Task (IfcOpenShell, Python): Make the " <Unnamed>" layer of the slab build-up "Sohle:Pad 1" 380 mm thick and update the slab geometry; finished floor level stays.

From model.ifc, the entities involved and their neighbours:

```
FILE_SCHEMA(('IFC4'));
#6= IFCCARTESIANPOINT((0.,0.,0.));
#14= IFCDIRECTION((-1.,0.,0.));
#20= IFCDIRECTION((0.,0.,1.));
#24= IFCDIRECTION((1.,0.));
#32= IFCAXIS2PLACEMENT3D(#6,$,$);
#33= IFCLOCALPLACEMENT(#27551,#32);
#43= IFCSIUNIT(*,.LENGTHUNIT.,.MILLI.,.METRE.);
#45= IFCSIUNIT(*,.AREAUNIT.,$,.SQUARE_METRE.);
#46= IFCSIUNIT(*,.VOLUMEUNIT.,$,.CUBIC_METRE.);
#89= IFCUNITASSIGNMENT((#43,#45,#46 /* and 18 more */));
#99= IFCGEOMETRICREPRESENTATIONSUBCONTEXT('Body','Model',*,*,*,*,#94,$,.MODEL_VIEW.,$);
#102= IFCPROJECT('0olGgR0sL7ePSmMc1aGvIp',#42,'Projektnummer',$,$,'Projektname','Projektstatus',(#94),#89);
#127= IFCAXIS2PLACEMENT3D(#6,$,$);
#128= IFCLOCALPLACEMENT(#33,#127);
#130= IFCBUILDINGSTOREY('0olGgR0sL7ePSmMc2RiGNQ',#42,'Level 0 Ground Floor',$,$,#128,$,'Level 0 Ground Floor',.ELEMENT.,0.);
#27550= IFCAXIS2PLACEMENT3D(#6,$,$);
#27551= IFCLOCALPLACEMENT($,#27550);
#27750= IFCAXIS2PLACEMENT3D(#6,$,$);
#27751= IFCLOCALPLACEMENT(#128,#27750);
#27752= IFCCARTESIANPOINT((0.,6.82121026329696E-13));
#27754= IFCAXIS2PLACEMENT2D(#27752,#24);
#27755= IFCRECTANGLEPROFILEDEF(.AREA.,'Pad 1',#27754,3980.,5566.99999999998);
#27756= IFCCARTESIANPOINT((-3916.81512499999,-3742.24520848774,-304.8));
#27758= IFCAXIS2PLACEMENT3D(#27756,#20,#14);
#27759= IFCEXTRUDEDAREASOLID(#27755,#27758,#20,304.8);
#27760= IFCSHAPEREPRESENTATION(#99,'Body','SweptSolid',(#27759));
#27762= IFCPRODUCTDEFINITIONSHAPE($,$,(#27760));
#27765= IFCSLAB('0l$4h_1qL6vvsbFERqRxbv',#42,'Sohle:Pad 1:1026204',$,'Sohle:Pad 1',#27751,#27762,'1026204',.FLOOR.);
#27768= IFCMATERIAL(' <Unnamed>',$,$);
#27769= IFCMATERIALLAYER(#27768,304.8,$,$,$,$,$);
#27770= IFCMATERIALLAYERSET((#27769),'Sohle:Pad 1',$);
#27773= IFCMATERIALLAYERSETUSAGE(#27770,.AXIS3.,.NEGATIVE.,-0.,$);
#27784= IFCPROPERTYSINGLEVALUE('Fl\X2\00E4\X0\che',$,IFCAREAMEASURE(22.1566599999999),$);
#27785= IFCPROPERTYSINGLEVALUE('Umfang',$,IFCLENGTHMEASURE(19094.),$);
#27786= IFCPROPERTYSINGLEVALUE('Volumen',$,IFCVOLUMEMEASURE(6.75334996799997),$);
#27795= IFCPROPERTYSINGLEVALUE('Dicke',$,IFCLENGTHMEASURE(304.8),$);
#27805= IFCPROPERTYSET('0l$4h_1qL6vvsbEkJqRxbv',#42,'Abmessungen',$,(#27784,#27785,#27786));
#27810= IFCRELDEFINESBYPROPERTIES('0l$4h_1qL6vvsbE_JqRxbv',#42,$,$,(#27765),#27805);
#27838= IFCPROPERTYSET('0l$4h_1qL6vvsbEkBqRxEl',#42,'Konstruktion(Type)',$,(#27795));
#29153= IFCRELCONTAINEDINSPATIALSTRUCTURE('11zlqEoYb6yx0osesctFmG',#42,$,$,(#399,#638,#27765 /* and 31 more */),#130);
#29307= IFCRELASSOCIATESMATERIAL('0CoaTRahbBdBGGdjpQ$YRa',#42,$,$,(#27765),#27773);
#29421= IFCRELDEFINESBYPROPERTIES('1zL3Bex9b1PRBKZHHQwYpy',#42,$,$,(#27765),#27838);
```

```python
import ifcopenshell
import ifcopenshell.api.pset
import ifcopenshell.util.element
import ifcopenshell.util.representation

model = ifcopenshell.open("model.ifc")

layer_set = model.by_id(27770)
layer = next(l for l in layer_set.MaterialLayers if l.Material and l.Material.Name == " <Unnamed>")
change = 380.0 - layer.LayerThickness
layer.LayerThickness += change

# Geometry does not follow the layer set by itself.
slabs = [e for e in ifcopenshell.util.element.get_elements_by_material(model, layer_set) if e.is_a("IfcSlab")]
for slab in sorted(slabs, key=lambda e: e.id()):
    body = ifcopenshell.util.representation.get_representation(slab, "Model", "Body")
    solid = body.Items[0]
    old_depth = solid.Depth
    solid.Depth += change
    # Extruded upwards: lower the start of the extrusion so the top stays.
    x, y, z = solid.Position.Location.Coordinates
    solid.Position.Location = model.createIfcCartesianPoint((x, y, z - change))
    pset = model.by_id(ifcopenshell.util.element.get_pset(slab, "Abmessungen", should_inherit=False)["id"])
    ifcopenshell.api.pset.edit_pset(model, pset=pset, properties={
        "Volumen": model.create_entity("IfcVolumeMeasure", ifcopenshell.util.element.get_pset(slab, "Abmessungen", "Volumen") * solid.Depth / old_depth),
    })
    pset = model.by_id(ifcopenshell.util.element.get_pset(slab, "Konstruktion(Type)", should_inherit=False)["id"])
    ifcopenshell.api.pset.edit_pset(model, pset=pset, properties={
        "Dicke": model.create_entity("IfcLengthMeasure", solid.Depth),
    })
    print(slab.id(), f"{old_depth:g} -> {solid.Depth:g}")

model.write("model-out.ifc")
```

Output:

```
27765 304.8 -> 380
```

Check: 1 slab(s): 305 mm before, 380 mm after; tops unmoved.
